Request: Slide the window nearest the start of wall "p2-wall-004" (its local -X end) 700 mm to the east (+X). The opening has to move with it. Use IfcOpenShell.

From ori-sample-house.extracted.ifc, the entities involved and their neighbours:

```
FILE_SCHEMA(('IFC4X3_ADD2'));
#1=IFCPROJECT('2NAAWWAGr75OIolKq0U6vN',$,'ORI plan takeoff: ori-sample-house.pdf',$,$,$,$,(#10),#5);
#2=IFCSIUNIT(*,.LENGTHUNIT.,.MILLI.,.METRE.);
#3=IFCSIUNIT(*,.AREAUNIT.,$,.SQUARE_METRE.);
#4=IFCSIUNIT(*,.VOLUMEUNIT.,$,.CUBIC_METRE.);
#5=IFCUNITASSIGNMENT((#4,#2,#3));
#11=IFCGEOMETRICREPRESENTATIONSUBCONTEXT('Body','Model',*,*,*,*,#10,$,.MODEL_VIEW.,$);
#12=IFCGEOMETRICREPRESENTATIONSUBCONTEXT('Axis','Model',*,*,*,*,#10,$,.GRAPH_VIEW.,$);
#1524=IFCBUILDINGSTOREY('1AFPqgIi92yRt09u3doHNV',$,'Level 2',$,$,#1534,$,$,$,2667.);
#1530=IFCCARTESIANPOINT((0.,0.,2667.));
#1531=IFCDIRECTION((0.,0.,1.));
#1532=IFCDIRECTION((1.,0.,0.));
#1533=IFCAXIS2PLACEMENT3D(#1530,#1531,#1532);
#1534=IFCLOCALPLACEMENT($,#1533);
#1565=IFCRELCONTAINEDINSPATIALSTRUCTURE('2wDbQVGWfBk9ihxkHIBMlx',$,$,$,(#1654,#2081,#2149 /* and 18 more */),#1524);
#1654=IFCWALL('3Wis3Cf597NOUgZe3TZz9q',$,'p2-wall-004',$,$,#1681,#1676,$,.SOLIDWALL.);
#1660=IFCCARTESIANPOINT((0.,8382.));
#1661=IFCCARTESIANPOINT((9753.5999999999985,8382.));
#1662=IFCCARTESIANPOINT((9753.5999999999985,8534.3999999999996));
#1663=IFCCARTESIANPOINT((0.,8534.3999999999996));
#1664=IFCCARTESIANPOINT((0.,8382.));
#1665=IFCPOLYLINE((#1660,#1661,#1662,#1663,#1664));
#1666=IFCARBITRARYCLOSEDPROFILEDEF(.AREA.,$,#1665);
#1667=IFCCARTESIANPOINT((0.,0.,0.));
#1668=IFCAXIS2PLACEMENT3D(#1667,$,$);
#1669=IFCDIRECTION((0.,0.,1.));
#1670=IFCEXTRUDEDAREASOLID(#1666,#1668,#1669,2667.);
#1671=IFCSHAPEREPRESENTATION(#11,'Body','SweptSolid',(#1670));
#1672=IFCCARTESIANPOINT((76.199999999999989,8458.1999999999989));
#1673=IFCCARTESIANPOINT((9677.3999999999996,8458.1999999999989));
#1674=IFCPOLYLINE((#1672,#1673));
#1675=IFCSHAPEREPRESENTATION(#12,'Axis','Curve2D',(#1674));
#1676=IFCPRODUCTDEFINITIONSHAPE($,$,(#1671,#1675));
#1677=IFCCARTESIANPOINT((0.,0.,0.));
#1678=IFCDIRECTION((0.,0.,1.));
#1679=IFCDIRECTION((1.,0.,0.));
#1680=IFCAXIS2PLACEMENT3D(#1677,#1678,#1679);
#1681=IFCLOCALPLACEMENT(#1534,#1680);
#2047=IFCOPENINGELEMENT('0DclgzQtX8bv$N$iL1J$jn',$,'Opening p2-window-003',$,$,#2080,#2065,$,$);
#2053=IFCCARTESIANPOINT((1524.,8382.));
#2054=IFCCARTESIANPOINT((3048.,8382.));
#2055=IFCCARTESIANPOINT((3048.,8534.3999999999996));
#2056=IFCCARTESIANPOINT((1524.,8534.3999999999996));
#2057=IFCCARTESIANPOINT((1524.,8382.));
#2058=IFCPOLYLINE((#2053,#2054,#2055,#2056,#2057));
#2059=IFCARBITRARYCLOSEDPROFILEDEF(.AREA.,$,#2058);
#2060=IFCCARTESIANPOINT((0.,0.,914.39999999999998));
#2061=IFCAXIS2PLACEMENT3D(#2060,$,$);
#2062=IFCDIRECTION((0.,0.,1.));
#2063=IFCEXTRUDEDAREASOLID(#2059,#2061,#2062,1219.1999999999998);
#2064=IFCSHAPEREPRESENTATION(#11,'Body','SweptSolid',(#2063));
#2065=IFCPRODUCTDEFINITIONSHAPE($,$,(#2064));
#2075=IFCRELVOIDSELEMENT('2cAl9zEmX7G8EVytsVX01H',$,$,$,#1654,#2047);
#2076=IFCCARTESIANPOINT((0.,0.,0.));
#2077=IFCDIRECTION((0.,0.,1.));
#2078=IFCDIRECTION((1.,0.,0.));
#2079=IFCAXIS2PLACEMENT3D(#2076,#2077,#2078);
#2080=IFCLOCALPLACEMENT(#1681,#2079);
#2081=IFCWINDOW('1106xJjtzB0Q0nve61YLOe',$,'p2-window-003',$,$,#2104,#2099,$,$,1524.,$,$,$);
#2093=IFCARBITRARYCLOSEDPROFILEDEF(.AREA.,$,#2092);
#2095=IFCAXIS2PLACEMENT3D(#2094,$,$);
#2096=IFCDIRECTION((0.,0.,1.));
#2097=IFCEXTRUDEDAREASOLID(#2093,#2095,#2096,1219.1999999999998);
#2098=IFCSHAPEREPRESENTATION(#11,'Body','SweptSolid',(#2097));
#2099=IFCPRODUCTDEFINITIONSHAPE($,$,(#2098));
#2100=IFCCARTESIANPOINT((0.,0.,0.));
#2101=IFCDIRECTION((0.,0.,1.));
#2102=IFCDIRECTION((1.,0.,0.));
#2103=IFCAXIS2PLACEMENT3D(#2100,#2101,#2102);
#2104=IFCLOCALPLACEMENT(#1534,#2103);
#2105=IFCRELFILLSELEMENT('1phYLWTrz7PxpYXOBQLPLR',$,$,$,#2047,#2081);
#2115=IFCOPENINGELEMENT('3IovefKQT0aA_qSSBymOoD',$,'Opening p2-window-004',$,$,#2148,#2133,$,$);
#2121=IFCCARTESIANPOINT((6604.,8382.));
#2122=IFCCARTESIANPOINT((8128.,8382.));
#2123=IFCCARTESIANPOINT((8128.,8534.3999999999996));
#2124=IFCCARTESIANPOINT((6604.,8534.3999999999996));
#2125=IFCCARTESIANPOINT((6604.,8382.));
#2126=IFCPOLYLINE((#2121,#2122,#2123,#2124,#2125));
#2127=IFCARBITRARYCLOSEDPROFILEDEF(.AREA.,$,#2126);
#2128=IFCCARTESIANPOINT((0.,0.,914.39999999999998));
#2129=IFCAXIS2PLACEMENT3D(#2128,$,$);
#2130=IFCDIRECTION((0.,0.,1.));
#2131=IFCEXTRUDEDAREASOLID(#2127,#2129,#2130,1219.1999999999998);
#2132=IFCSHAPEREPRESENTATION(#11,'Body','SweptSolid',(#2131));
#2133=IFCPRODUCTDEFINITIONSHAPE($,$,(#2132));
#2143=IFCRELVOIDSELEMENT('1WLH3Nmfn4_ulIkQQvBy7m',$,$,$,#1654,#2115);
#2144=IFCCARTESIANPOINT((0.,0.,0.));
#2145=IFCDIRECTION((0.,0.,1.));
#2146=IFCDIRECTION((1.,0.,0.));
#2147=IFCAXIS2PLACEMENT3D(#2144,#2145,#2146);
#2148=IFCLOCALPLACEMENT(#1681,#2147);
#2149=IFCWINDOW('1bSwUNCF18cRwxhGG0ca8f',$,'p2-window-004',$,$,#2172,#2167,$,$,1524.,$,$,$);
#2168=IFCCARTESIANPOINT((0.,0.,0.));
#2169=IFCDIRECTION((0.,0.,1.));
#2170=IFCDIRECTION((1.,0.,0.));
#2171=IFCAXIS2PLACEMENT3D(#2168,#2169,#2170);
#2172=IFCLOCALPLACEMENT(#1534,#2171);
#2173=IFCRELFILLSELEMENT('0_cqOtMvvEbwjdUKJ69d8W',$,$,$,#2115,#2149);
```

```python
import ifcopenshell
import ifcopenshell.api.geometry
import ifcopenshell.util.placement
import ifcopenshell.util.unit

model = ifcopenshell.open("ori-sample-house.extracted.ifc")
unit_scale = ifcopenshell.util.unit.calculate_unit_scale(model)

window = model.by_guid("1106xJjtzB0Q0nve61YLOe")
opening = window.FillsVoids[0].RelatingOpeningElement
wall = opening.VoidsElements[0].RelatingBuildingElement

wall_matrix = ifcopenshell.util.placement.get_local_placement(wall.ObjectPlacement)
shift = wall_matrix[:3, 0] * 0.7 / unit_scale
before = ifcopenshell.util.placement.get_local_placement(window.ObjectPlacement)[:3, 3].copy()

# The window is not placed relative to its opening, so move both.
for product in (opening, window):
    matrix = ifcopenshell.util.placement.get_local_placement(product.ObjectPlacement)
    matrix[:3, 3] += shift
    ifcopenshell.api.geometry.edit_object_placement(model, product=product, matrix=matrix, is_si=False)

after = ifcopenshell.util.placement.get_local_placement(window.ObjectPlacement)[:3, 3]
print("window moved by", (after - before).round(3) + 0.0)

model.write("ori-sample-house.extracted_rev.ifc")
```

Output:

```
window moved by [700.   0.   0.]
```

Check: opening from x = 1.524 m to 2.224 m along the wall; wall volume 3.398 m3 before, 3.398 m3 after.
